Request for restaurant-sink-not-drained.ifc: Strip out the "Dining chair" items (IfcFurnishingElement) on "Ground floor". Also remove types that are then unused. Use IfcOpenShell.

First a look at what the model holds.

```python
import ifcopenshell
import ifcopenshell.util.element

model = ifcopenshell.open("restaurant-sink-not-drained.ifc")
print(model.schema)
storey = next(s for s in model.by_type("IfcBuildingStorey") if s.Name == "Ground floor")
furniture = [e for e in ifcopenshell.util.element.get_decomposition(storey) if e.is_a("IfcFurnishingElement")]
seen = {}
for e in furniture:
    element_type = ifcopenshell.util.element.get_type(e)
    name = element_type.Name if element_type not in (None, e) else None
    seen[name] = seen.get(name, 0) + 1
for name, count in sorted(seen.items(), key=str):
    print(count, "x", name)
```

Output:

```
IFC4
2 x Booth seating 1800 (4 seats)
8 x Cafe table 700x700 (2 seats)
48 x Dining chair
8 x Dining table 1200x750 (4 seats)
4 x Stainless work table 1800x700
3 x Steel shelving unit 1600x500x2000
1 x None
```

```python
import ifcopenshell
import ifcopenshell.api.root
import ifcopenshell.util.element

model = ifcopenshell.open("restaurant-sink-not-drained.ifc")

storey = next(s for s in model.by_type("IfcBuildingStorey") if s.Name == "Ground floor")
furniture = [e for e in ifcopenshell.util.element.get_decomposition(storey) if e.is_a("IfcFurnishingElement")]
targets = [e for e in furniture if (t := ifcopenshell.util.element.get_type(e)) not in (None, e) and t.Name == "Dining chair"]
types = {ifcopenshell.util.element.get_type(e) for e in targets} - {None, *targets}

for e in targets:
    ifcopenshell.api.root.remove_product(model, product=e)
print(len(targets), "removed")

unused = [t for t in types if not ifcopenshell.util.element.get_types(t)]
for t in unused:
    ifcopenshell.api.root.remove_product(model, product=t)
print(len(unused), "unused types removed")

model.write("restaurant-sink-not-drained-out.ifc")
```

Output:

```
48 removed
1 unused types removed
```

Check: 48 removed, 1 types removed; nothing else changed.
